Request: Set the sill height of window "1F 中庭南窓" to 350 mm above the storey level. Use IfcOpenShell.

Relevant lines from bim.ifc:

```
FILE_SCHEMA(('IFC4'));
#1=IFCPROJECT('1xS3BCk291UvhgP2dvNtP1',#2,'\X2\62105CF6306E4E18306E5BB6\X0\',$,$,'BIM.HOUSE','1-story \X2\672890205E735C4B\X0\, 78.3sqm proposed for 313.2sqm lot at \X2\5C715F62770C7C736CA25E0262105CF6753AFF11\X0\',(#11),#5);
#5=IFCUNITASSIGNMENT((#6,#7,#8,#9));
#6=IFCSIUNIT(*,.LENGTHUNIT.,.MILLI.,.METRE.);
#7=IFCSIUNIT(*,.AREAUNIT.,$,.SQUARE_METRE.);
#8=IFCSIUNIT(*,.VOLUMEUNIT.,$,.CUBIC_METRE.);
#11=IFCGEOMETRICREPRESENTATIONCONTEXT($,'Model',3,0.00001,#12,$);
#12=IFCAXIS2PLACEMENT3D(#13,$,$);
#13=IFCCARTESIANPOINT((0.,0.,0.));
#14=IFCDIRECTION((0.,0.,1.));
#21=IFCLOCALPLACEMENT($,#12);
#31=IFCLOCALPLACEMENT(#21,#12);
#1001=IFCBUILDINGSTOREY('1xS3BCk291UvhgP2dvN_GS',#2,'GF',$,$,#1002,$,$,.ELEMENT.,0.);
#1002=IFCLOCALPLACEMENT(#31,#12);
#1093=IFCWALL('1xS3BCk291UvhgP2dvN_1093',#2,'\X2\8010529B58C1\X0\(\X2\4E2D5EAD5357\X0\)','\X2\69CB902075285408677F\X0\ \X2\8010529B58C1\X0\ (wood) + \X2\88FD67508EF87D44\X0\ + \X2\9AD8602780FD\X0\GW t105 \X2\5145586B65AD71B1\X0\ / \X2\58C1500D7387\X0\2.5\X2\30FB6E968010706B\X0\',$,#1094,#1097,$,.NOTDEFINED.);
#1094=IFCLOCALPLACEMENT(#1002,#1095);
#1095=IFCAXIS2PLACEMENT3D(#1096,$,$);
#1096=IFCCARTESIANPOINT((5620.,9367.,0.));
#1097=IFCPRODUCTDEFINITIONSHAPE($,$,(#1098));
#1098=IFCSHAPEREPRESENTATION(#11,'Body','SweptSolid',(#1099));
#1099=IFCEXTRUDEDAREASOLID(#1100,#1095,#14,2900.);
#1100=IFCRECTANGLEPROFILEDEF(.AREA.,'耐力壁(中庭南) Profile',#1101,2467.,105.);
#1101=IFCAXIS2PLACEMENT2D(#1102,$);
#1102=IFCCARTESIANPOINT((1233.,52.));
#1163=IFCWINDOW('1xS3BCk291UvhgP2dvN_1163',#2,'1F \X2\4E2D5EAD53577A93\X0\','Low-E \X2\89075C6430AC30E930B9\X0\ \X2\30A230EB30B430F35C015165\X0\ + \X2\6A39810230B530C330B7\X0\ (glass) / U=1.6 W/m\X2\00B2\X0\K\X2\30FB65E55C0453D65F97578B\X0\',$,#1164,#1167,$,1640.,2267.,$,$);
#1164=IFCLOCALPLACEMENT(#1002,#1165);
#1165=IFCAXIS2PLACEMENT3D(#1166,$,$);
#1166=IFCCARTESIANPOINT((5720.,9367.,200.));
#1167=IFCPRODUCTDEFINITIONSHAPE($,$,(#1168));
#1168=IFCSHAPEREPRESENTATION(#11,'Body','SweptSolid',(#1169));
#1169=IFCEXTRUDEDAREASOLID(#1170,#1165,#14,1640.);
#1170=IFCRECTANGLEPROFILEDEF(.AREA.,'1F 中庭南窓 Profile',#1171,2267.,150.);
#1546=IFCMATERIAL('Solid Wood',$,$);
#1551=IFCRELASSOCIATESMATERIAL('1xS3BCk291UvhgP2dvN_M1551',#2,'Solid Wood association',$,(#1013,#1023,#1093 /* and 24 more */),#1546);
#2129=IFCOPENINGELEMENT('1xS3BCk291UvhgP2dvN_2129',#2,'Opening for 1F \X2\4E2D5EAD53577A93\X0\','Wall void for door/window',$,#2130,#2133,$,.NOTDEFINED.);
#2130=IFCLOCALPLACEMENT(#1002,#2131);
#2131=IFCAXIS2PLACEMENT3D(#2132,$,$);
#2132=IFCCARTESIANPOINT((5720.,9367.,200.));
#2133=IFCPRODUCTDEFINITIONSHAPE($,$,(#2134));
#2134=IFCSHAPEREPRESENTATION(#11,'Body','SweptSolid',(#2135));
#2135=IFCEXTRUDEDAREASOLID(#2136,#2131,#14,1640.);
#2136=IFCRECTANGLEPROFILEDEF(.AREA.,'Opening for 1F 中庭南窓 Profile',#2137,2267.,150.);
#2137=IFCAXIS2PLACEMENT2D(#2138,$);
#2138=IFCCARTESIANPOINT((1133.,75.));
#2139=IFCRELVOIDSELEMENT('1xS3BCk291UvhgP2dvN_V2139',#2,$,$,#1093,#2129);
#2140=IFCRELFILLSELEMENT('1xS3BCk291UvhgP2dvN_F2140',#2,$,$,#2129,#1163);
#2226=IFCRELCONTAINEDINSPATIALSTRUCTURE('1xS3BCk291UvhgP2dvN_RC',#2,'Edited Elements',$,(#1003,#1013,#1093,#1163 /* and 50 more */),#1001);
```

```python
import numpy as np
import ifcopenshell
import ifcopenshell.api.geometry
import ifcopenshell.geom
import ifcopenshell.util.element
import ifcopenshell.util.placement
import ifcopenshell.util.shape
import ifcopenshell.util.unit

model = ifcopenshell.open("bim.ifc")
unit_scale = ifcopenshell.util.unit.calculate_unit_scale(model)

window = model.by_guid("1xS3BCk291UvhgP2dvN_1163")
opening = window.FillsVoids[0].RelatingOpeningElement
storey = ifcopenshell.util.element.get_container(window, ifc_class="IfcBuildingStorey")
level = ifcopenshell.util.placement.get_local_placement(storey.ObjectPlacement)[2, 3]

# The opening's origin need not be at the sill, so measure its lowest point.
shape = ifcopenshell.geom.create_shape(ifcopenshell.geom.settings(), opening)
bottom = ifcopenshell.util.shape.get_shape_bottom_elevation(shape, shape.geometry) / unit_scale
dz = level + 350.0 - bottom

shift = np.array([0.0, 0.0, dz])
# The window is not placed relative to its opening, so move both.
for product in (opening, window):
    matrix = ifcopenshell.util.placement.get_local_placement(product.ObjectPlacement)
    matrix[:3, 3] += shift
    ifcopenshell.api.geometry.edit_object_placement(model, product=product, matrix=matrix, is_si=False)

print(f"moved by {dz * unit_scale:+.3f} m")

model.write("bim_v2.ifc")
```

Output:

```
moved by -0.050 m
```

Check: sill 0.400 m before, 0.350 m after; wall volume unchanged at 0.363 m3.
